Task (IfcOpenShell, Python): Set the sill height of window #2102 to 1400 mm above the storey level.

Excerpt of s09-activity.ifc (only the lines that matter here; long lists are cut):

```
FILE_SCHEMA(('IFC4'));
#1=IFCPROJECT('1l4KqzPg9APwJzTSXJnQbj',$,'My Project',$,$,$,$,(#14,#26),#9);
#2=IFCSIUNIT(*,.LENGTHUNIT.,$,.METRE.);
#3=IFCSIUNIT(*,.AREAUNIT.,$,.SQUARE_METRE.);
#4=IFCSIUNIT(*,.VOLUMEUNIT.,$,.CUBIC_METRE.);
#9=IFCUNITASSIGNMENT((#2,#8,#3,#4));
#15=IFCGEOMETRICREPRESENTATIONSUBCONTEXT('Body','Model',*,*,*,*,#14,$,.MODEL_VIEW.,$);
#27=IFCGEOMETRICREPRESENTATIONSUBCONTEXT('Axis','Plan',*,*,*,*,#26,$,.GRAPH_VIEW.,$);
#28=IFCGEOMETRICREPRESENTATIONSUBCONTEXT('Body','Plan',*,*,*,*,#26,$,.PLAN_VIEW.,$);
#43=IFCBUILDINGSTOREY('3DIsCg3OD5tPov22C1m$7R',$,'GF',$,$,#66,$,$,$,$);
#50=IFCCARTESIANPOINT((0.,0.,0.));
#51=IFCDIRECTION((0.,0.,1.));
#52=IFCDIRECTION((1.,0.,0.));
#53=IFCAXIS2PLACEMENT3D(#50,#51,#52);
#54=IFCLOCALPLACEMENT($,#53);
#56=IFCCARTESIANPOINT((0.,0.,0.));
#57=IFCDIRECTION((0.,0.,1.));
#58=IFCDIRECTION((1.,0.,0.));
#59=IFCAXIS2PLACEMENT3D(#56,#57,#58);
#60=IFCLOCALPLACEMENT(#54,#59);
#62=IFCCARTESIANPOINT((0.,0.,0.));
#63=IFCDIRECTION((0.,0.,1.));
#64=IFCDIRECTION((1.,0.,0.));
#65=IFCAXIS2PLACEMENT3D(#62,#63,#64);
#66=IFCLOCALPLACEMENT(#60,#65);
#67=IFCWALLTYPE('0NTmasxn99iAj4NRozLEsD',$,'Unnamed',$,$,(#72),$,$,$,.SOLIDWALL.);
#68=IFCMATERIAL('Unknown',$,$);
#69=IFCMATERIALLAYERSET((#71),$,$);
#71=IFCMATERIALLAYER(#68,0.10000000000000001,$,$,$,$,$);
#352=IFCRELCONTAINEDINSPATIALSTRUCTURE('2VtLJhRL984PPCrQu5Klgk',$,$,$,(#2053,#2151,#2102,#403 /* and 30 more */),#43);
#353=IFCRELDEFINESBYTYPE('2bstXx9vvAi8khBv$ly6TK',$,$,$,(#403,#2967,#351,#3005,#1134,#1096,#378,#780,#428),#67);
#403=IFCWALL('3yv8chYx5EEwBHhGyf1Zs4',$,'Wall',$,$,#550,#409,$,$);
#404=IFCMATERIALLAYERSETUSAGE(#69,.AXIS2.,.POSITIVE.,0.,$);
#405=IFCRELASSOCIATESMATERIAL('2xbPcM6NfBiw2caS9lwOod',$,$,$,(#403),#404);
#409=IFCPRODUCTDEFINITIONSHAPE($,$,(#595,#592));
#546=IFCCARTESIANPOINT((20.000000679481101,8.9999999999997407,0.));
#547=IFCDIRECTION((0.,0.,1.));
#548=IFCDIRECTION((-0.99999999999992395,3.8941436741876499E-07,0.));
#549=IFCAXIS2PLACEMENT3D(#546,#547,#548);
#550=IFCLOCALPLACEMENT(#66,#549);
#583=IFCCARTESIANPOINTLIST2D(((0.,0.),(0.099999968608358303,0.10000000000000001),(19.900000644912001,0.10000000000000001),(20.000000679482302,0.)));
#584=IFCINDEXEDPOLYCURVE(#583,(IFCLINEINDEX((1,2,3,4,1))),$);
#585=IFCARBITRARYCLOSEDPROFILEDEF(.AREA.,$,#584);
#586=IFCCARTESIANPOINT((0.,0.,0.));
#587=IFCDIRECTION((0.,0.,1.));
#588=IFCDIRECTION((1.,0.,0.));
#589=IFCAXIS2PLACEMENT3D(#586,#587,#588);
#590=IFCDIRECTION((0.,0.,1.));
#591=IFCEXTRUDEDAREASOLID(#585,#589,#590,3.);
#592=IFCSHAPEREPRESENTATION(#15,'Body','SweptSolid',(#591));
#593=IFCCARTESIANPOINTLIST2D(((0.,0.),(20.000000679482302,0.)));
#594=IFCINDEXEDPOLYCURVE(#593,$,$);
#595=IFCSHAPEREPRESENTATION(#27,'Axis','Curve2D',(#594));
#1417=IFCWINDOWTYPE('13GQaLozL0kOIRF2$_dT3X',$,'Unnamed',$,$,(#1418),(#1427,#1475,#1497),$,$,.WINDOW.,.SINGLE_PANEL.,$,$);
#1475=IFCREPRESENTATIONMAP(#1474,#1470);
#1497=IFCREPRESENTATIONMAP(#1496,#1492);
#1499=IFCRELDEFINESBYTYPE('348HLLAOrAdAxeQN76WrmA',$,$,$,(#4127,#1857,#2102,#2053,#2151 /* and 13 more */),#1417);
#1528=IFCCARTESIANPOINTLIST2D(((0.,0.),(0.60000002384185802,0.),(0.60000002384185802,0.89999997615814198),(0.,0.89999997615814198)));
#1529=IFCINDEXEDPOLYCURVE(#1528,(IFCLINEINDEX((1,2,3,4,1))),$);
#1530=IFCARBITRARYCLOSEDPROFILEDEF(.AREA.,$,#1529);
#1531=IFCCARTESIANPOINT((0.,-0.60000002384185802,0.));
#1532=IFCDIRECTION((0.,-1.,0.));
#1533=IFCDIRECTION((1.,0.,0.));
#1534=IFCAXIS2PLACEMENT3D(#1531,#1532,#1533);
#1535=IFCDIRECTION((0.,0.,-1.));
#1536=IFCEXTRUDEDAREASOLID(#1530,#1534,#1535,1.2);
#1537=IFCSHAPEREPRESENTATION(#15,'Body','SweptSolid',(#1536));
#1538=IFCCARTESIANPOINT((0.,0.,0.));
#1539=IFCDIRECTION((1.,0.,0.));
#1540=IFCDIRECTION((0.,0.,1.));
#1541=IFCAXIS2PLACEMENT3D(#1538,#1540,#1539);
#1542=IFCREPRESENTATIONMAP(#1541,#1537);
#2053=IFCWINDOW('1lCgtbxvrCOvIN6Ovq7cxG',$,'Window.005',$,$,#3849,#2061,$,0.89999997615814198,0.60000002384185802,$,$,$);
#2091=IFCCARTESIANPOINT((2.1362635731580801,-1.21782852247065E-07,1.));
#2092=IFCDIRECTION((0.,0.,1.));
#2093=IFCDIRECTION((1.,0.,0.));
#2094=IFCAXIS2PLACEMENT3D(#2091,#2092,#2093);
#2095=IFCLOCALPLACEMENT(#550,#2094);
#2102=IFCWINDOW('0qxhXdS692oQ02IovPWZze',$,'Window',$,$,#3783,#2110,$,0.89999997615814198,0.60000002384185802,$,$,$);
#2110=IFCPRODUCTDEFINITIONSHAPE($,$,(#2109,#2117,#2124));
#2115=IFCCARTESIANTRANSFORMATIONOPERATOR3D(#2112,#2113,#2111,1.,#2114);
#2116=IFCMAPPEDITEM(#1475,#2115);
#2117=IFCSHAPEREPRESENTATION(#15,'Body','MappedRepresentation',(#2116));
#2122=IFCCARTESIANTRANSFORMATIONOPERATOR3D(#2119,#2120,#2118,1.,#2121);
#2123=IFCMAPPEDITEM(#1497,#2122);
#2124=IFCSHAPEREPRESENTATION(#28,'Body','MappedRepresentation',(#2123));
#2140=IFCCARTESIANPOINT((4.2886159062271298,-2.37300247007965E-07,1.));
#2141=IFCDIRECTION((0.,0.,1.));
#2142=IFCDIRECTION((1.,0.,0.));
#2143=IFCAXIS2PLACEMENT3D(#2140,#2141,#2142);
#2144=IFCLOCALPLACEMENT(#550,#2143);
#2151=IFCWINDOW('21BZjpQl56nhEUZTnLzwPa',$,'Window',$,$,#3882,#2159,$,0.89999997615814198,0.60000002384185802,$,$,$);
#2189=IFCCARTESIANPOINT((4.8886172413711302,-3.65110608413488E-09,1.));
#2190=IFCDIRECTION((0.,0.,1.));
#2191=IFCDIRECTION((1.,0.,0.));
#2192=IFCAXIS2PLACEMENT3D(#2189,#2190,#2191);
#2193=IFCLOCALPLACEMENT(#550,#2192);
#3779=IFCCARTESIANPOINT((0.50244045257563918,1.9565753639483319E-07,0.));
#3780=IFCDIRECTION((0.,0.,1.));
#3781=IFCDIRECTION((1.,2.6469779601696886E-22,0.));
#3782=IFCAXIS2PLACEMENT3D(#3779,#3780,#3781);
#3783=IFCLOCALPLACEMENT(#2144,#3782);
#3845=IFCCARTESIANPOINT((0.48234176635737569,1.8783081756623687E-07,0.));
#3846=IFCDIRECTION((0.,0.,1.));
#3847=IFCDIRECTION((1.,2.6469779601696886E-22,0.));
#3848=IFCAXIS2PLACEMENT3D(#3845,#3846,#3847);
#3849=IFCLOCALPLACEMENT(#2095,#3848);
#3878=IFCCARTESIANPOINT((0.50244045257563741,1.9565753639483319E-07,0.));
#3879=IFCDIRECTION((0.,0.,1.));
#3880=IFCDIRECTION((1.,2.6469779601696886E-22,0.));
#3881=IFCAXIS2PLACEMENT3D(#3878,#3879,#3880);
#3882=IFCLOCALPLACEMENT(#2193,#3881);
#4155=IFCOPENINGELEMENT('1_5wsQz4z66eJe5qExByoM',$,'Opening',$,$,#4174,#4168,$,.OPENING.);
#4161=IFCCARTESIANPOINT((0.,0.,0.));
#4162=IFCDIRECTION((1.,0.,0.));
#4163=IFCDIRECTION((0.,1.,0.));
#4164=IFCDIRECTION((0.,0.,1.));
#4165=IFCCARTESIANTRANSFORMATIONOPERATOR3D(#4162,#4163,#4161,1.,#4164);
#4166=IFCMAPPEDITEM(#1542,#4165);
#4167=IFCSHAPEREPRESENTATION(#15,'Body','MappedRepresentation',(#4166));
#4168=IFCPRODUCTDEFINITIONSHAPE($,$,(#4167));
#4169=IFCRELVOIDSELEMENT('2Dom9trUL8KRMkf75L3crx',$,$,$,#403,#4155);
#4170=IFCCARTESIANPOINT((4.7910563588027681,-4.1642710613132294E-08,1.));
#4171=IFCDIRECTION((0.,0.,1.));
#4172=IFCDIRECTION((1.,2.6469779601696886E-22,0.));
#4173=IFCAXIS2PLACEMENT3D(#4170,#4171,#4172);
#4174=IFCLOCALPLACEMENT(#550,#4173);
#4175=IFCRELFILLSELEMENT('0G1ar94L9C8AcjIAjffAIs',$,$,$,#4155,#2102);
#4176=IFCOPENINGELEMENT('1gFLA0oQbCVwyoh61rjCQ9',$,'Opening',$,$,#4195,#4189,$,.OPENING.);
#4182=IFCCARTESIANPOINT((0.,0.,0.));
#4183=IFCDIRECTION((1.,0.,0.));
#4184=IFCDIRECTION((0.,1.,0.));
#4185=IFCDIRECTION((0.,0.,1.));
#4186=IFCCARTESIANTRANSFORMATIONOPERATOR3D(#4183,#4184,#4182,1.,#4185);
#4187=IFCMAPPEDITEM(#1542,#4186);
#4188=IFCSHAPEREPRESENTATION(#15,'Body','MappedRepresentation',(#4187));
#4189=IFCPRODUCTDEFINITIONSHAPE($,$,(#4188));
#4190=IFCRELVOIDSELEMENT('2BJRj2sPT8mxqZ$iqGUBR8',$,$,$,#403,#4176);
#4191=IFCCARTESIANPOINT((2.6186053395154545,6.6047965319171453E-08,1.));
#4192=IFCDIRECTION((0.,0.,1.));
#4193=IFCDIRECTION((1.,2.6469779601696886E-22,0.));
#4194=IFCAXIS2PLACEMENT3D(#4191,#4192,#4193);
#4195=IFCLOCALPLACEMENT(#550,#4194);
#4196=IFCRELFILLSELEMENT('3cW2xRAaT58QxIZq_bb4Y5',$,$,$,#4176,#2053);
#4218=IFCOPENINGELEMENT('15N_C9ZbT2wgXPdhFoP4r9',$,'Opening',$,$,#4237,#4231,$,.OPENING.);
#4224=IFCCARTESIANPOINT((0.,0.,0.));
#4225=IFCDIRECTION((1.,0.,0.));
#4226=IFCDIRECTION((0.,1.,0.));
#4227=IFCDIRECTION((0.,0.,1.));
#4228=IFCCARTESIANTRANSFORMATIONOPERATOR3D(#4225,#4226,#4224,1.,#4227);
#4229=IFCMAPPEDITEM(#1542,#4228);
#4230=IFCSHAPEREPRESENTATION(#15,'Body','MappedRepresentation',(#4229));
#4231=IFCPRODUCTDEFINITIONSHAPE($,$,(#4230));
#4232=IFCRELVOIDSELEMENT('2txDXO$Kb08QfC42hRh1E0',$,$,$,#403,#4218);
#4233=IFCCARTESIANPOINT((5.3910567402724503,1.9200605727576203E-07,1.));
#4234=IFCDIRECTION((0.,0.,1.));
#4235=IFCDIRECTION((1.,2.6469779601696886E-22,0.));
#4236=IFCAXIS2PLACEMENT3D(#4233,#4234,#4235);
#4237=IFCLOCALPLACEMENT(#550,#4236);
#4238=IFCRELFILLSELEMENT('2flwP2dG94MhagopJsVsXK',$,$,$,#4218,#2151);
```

```python
import numpy as np
import ifcopenshell
import ifcopenshell.api.geometry
import ifcopenshell.geom
import ifcopenshell.util.element
import ifcopenshell.util.placement
import ifcopenshell.util.shape
import ifcopenshell.util.unit

model = ifcopenshell.open("s09-activity.ifc")
unit_scale = ifcopenshell.util.unit.calculate_unit_scale(model)

window = model.by_guid("0qxhXdS692oQ02IovPWZze")
opening = window.FillsVoids[0].RelatingOpeningElement
storey = ifcopenshell.util.element.get_container(window, ifc_class="IfcBuildingStorey")
level = ifcopenshell.util.placement.get_local_placement(storey.ObjectPlacement)[2, 3]

# The opening's origin need not be at the sill, so measure its lowest point.
shape = ifcopenshell.geom.create_shape(ifcopenshell.geom.settings(), opening)
bottom = ifcopenshell.util.shape.get_shape_bottom_elevation(shape, shape.geometry) / unit_scale
dz = level + 1.4 - bottom

shift = np.array([0.0, 0.0, dz])
# The window is not placed relative to its opening, so move both.
for product in (opening, window):
    matrix = ifcopenshell.util.placement.get_local_placement(product.ObjectPlacement)
    matrix[:3, 3] += shift
    ifcopenshell.api.geometry.edit_object_placement(model, product=product, matrix=matrix, is_si=False)

print(f"moved by {dz * unit_scale:+.3f} m")

model.write("s09-activity_edited.ifc")
```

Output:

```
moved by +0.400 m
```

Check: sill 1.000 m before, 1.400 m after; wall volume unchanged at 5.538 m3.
